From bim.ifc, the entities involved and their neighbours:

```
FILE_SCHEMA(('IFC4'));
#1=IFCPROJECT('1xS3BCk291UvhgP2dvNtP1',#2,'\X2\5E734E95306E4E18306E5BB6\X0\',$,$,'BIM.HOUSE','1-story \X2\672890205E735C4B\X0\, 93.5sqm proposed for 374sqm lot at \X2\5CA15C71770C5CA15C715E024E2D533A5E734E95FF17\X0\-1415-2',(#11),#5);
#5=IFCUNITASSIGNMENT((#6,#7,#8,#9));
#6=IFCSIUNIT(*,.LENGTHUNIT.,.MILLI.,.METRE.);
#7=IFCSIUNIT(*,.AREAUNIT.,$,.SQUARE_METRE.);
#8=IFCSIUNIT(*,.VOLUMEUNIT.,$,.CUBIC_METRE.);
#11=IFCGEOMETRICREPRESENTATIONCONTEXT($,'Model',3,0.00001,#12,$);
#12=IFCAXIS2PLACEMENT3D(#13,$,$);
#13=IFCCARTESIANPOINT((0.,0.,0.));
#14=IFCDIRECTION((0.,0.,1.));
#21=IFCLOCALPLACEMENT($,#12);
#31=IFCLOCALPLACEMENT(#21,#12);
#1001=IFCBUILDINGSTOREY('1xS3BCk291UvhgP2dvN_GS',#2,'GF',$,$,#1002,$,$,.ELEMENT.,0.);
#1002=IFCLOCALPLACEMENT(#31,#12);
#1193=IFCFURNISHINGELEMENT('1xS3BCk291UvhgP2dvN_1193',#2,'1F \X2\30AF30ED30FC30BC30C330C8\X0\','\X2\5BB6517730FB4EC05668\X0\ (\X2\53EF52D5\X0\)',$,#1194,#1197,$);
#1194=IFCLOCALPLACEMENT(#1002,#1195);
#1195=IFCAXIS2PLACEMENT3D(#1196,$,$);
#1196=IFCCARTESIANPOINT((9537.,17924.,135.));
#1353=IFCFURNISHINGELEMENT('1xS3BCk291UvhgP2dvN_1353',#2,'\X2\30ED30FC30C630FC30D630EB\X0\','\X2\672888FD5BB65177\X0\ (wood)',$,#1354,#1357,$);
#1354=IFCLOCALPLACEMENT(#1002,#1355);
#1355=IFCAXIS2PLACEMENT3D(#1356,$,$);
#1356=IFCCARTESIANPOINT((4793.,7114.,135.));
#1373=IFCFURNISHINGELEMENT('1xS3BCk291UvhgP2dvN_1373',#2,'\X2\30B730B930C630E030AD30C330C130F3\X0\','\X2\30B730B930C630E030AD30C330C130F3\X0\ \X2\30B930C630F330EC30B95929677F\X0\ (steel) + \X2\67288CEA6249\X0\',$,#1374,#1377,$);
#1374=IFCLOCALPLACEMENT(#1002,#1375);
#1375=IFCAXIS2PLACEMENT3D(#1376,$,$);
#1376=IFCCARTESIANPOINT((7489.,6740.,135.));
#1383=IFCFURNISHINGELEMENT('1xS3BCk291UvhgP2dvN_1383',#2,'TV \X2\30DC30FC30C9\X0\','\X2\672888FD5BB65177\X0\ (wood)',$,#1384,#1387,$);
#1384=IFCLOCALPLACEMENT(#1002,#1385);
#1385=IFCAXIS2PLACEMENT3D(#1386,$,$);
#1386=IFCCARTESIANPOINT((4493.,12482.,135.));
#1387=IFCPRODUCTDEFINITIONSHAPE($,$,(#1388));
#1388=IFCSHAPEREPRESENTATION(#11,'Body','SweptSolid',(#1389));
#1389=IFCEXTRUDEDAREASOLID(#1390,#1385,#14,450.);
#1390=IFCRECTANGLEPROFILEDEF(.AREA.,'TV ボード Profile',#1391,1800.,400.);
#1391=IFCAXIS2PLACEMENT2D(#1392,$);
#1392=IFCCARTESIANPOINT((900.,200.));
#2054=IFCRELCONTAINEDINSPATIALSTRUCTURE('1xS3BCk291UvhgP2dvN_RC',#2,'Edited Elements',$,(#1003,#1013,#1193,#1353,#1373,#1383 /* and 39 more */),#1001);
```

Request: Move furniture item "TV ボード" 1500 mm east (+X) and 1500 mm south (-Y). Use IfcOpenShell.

```python
import ifcopenshell
import ifcopenshell.api.geometry
import ifcopenshell.util.placement
import ifcopenshell.util.unit

model = ifcopenshell.open("bim.ifc")
unit_scale = ifcopenshell.util.unit.calculate_unit_scale(model)

item = model.by_guid("1xS3BCk291UvhgP2dvN_1383")
matrix = ifcopenshell.util.placement.get_local_placement(item.ObjectPlacement)
matrix[0, 3] += 1.5 / unit_scale
matrix[1, 3] -= 1.5 / unit_scale
ifcopenshell.api.geometry.edit_object_placement(model, product=item, matrix=matrix, is_si=False)

print(ifcopenshell.util.placement.get_local_placement(item.ObjectPlacement).round(3) + 0.0)

model.write("bim_rev.ifc")
```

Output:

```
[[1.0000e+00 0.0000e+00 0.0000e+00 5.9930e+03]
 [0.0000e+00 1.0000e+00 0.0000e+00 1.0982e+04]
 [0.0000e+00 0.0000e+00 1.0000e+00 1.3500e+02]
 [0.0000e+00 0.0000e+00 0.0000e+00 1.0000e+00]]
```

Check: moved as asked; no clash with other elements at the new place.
